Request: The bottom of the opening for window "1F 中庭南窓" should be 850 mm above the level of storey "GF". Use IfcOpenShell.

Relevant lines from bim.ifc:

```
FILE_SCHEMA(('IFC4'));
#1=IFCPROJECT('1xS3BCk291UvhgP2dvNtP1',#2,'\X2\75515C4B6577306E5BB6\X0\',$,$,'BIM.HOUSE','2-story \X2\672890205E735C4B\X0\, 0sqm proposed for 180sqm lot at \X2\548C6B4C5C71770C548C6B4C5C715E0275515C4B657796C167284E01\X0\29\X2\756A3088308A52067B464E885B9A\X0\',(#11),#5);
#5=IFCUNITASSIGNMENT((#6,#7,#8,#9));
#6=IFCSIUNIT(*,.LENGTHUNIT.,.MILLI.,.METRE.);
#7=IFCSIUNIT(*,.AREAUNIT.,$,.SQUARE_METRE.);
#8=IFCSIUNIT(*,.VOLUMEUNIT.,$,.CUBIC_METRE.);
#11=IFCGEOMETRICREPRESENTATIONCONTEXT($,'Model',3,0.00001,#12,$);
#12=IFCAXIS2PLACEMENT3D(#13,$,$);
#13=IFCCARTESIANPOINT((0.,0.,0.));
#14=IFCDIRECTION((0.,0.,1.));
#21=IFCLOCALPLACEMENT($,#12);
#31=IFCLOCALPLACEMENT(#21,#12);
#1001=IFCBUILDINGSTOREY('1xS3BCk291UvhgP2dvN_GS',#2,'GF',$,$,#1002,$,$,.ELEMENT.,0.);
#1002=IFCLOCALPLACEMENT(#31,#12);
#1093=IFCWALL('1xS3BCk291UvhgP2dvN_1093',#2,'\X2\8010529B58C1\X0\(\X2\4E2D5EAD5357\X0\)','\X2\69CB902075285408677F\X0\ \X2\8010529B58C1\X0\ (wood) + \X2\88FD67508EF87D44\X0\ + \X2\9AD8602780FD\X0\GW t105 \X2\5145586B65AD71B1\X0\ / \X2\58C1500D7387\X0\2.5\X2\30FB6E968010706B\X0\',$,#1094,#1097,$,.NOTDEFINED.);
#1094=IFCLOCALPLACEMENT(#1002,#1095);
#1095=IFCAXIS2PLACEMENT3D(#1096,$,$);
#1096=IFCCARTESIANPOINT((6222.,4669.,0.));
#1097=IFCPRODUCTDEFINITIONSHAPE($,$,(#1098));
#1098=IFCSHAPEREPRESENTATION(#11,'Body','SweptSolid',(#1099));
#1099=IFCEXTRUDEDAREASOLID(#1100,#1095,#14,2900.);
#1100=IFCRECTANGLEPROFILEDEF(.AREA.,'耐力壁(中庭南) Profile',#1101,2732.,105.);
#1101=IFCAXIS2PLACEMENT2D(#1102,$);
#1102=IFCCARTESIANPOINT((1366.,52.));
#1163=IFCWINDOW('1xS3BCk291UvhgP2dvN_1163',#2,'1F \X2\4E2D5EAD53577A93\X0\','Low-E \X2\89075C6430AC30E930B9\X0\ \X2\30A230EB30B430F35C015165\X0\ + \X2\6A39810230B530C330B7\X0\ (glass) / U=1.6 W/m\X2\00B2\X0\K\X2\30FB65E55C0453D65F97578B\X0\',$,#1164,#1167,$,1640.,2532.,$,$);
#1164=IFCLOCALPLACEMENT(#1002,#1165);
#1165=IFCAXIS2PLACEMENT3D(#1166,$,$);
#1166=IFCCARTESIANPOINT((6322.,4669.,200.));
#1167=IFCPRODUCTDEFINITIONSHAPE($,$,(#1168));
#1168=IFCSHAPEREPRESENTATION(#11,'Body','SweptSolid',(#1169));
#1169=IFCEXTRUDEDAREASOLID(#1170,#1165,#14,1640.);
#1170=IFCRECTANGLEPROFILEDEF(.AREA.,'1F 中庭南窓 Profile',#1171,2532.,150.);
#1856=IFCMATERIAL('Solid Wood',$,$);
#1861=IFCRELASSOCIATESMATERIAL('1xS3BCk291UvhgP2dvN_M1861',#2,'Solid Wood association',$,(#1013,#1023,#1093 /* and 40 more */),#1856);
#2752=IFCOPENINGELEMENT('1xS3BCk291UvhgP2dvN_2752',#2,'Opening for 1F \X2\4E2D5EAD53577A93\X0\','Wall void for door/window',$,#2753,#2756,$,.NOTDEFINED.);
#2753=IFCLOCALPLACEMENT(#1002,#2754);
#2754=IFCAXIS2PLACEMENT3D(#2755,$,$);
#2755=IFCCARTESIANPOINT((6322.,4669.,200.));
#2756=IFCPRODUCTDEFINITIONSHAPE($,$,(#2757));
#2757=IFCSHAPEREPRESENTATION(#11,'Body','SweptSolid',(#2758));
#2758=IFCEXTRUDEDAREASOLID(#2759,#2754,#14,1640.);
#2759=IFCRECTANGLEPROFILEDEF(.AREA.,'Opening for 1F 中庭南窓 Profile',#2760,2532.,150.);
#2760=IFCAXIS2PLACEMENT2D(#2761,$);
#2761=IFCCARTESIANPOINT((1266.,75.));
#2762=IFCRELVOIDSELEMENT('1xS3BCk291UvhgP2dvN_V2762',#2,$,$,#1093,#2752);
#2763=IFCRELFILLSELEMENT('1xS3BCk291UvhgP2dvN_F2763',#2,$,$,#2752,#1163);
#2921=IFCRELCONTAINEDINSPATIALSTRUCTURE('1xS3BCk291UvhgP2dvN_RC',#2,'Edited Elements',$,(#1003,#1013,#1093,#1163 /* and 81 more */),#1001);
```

```python
import numpy as np
import ifcopenshell
import ifcopenshell.api.geometry
import ifcopenshell.geom
import ifcopenshell.util.element
import ifcopenshell.util.placement
import ifcopenshell.util.shape
import ifcopenshell.util.unit

model = ifcopenshell.open("bim.ifc")
unit_scale = ifcopenshell.util.unit.calculate_unit_scale(model)

window = model.by_guid("1xS3BCk291UvhgP2dvN_1163")
opening = window.FillsVoids[0].RelatingOpeningElement
storey = ifcopenshell.util.element.get_container(window, ifc_class="IfcBuildingStorey")
level = ifcopenshell.util.placement.get_local_placement(storey.ObjectPlacement)[2, 3]

# The opening's origin need not be at the sill, so measure its lowest point.
shape = ifcopenshell.geom.create_shape(ifcopenshell.geom.settings(), opening)
bottom = ifcopenshell.util.shape.get_shape_bottom_elevation(shape, shape.geometry) / unit_scale
dz = level + 0.85 / unit_scale - bottom

shift = np.array([0.0, 0.0, dz])
# The window is not placed relative to its opening, so move both.
for product in (opening, window):
    matrix = ifcopenshell.util.placement.get_local_placement(product.ObjectPlacement)
    matrix[:3, 3] += shift
    ifcopenshell.api.geometry.edit_object_placement(model, product=product, matrix=matrix, is_si=False)

print(f"moved by {dz * unit_scale:+.3f} m")

model.write("bim_rev.ifc")
```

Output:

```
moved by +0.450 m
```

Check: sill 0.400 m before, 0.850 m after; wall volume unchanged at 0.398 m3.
